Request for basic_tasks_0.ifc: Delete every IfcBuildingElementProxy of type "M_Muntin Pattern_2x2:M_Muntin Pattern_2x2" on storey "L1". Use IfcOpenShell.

First a look at what the model holds.

```python
import ifcopenshell
import ifcopenshell.util.element

model = ifcopenshell.open("basic_tasks_0.ifc")
print(model.schema)
storey = next(s for s in model.by_type("IfcBuildingStorey") if s.Name == "L1")
proxies = [e for e in ifcopenshell.util.element.get_decomposition(storey) if e.is_a("IfcBuildingElementProxy")]
seen = {}
for e in proxies:
    element_type = ifcopenshell.util.element.get_type(e)
    name = element_type.Name if element_type not in (None, e) else None
    seen[name] = seen.get(name, 0) + 1
for name, count in sorted(seen.items(), key=str):
    print(count, "x", name)
```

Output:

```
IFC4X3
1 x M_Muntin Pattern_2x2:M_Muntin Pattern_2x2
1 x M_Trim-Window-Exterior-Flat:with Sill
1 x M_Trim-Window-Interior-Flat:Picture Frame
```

```python
import ifcopenshell
import ifcopenshell.api.root
import ifcopenshell.util.element

model = ifcopenshell.open("basic_tasks_0.ifc")

storey = next(s for s in model.by_type("IfcBuildingStorey") if s.Name == "L1")
proxies = [e for e in ifcopenshell.util.element.get_decomposition(storey) if e.is_a("IfcBuildingElementProxy")]
targets = [e for e in proxies if (t := ifcopenshell.util.element.get_type(e)) not in (None, e) and t.Name == "M_Muntin Pattern_2x2:M_Muntin Pattern_2x2"]

for e in targets:
    ifcopenshell.api.root.remove_product(model, product=e)
print(len(targets), "removed")

model.write("basic_tasks_0_edited.ifc")
```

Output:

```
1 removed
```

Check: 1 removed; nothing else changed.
